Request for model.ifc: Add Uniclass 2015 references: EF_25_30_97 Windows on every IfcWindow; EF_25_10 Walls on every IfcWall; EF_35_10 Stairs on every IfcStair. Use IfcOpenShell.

First a look at what the model holds.

```python
import ifcopenshell

model = ifcopenshell.open("model.ifc")
print(model.schema)
print("classifications:", [c.Name for c in model.by_type("IfcClassification")])
for ifc_class in ("IfcDoor", "IfcRoof", "IfcStair", "IfcWall", "IfcWindow"):
    print(ifc_class, len(model.by_type(ifc_class)))
```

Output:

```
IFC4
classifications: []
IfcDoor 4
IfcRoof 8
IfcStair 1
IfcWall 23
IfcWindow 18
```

```python
import ifcopenshell
import ifcopenshell.api.classification

model = ifcopenshell.open("model.ifc")

system = ifcopenshell.api.classification.add_classification(model, classification="Uniclass 2015")

codes = {
    "IfcWindow": ("EF_25_30_97", "Windows"),
    "IfcWall": ("EF_25_10", "Walls"),
    "IfcStair": ("EF_35_10", "Stairs"),
}
for ifc_class, (code, name) in codes.items():
    products = model.by_type(ifc_class)
    ifcopenshell.api.classification.add_reference(
        model, products=products, classification=system, identification=code, name=name
    )
    print(code, len(products))

model.write("model_rev.ifc")
```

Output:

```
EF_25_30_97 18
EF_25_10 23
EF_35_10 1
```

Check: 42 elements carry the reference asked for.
